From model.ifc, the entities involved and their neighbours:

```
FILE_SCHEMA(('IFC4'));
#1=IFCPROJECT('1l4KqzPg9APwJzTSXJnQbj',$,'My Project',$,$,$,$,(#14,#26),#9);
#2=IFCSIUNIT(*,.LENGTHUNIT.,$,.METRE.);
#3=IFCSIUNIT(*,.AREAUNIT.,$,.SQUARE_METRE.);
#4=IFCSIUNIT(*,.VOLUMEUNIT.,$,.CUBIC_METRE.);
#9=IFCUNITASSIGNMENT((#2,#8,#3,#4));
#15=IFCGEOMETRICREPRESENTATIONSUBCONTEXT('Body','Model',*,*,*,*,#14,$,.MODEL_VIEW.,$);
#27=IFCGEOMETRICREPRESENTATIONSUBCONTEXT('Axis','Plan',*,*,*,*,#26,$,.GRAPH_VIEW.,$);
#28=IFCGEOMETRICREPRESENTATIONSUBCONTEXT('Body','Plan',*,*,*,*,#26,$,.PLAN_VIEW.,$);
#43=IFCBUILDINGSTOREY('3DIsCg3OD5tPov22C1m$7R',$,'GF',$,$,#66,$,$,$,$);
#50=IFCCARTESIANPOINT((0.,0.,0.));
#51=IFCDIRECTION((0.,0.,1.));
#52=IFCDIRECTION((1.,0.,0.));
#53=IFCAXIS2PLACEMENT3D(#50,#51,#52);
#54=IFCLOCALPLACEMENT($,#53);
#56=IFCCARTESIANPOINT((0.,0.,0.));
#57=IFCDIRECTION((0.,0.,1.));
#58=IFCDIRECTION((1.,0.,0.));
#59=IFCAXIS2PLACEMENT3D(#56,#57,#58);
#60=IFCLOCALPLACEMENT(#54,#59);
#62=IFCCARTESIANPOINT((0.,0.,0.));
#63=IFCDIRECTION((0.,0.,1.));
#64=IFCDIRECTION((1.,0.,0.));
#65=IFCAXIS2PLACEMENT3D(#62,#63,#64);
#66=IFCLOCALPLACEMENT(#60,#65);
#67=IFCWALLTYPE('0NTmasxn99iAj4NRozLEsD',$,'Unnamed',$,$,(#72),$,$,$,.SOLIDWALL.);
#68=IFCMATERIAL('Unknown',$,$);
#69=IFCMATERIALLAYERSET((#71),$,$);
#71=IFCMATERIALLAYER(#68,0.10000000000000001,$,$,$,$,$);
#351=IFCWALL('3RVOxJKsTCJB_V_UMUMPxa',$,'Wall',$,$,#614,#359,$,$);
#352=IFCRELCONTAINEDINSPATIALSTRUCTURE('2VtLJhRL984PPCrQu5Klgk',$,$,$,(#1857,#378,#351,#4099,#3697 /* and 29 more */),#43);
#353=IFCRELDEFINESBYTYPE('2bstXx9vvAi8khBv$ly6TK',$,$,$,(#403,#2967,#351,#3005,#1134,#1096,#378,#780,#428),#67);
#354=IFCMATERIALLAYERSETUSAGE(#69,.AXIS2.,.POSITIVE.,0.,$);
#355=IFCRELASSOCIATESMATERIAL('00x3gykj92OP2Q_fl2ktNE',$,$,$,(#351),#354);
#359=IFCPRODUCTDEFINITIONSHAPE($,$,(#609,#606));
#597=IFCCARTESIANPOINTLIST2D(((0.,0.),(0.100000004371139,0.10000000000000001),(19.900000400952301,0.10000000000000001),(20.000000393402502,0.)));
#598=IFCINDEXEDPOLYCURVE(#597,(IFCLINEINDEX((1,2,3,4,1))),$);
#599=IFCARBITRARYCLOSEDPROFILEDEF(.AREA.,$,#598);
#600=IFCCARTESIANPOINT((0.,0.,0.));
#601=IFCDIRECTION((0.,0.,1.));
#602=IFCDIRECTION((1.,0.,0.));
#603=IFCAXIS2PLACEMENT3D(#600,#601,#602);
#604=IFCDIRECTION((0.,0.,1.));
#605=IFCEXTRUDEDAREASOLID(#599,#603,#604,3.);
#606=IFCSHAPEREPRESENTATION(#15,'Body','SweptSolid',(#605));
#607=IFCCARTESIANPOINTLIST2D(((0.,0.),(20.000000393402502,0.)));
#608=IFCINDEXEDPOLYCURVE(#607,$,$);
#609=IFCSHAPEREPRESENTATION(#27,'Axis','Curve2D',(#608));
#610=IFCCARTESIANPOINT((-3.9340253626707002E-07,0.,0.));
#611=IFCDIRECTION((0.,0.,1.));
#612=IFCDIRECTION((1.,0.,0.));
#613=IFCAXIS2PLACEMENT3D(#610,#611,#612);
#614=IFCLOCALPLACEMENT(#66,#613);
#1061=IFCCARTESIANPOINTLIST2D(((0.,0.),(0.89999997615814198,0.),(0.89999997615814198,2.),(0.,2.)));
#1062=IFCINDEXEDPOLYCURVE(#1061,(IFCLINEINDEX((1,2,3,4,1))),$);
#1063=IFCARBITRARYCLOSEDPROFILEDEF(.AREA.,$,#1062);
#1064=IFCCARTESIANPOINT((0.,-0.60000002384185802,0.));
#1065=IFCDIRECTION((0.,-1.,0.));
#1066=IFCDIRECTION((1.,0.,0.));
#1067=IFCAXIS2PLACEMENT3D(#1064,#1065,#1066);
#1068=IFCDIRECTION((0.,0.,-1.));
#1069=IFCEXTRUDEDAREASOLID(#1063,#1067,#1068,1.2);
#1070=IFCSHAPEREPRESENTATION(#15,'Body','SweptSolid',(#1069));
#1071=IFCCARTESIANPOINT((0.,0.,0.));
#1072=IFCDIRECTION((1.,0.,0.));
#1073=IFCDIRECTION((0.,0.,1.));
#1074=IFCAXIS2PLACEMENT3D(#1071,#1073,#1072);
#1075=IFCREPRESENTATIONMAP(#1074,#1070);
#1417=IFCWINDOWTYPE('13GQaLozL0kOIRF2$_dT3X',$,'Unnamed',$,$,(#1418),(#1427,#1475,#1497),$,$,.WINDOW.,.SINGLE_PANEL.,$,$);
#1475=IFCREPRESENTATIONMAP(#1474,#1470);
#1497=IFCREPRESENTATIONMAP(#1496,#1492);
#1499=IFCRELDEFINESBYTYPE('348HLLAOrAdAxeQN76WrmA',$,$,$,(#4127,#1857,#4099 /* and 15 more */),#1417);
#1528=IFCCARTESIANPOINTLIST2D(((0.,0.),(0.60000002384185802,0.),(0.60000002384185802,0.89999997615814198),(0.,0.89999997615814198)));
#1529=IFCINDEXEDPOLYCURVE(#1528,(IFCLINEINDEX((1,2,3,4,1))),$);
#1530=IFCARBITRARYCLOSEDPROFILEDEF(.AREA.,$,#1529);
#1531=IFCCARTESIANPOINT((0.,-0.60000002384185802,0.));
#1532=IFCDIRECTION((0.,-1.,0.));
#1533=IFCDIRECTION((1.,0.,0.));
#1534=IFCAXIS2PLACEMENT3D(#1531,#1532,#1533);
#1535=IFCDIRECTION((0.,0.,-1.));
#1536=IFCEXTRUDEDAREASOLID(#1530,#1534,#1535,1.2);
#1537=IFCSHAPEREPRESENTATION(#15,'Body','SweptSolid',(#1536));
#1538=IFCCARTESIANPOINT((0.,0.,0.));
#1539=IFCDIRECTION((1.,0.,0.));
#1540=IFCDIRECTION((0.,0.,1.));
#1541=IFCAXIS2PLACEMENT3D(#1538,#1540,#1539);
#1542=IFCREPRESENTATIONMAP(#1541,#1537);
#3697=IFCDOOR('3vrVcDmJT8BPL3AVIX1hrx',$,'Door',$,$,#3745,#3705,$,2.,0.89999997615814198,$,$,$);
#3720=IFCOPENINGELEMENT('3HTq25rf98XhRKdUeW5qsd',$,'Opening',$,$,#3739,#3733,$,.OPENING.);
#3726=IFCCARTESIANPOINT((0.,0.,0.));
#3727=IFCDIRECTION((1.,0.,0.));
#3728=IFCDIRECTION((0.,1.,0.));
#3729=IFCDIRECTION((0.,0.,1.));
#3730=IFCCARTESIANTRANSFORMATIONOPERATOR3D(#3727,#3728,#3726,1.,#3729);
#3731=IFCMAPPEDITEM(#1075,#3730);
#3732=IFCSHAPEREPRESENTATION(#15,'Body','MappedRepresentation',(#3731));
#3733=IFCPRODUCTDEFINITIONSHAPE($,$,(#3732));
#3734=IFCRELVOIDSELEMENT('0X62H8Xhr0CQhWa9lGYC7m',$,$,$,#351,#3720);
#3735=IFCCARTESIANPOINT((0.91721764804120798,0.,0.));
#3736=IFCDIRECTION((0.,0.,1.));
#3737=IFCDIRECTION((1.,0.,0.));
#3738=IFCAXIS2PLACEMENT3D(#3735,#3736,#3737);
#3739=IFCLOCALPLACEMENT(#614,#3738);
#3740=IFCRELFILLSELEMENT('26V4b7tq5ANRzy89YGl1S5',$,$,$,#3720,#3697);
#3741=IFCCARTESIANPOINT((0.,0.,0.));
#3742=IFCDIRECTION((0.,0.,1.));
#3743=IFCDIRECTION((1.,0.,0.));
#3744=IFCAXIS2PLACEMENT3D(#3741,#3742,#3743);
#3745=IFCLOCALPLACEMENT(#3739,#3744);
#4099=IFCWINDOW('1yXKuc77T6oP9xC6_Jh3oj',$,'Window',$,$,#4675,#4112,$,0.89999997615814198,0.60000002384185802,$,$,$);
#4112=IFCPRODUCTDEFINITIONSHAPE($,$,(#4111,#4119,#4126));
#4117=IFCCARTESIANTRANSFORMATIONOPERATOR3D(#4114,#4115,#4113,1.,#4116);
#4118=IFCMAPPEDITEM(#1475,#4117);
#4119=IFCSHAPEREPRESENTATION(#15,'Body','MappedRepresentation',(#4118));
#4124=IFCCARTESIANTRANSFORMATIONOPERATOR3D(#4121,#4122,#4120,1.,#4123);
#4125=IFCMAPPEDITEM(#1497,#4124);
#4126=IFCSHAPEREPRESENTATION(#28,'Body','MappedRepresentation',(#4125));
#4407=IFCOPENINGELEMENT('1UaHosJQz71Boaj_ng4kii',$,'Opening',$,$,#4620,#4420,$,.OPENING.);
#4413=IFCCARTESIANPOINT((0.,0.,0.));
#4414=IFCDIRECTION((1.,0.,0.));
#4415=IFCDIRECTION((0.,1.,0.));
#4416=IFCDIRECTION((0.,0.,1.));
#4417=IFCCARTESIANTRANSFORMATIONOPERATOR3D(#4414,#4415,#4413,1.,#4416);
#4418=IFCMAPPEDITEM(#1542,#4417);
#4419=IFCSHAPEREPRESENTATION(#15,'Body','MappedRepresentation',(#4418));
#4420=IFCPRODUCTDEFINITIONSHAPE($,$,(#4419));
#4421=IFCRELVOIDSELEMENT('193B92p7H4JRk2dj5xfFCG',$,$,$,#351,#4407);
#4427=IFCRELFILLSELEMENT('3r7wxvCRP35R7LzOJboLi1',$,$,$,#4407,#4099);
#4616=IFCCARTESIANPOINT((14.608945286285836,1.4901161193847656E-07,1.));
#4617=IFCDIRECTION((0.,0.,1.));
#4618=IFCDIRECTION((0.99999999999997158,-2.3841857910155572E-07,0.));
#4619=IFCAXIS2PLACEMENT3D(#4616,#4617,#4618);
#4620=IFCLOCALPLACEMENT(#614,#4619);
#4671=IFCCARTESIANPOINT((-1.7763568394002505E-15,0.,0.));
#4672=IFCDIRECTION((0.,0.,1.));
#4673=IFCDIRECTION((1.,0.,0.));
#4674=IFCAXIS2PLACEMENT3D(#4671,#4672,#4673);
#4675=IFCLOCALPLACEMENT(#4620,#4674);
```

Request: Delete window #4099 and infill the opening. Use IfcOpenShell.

```python
import ifcopenshell
import ifcopenshell.api.feature
import ifcopenshell.api.root
import ifcopenshell.geom
import ifcopenshell.util.shape

model = ifcopenshell.open("model.ifc")
settings = ifcopenshell.geom.settings()


def volume(element):
    """Net volume in cubic metres, openings subtracted."""
    shape = ifcopenshell.geom.create_shape(settings, element)
    return ifcopenshell.util.shape.get_volume(shape.geometry)


window = model.by_guid("1yXKuc77T6oP9xC6_Jh3oj")
opening = window.FillsVoids[0].RelatingOpeningElement
wall = opening.VoidsElements[0].RelatingBuildingElement
before = volume(wall)

ifcopenshell.api.root.remove_product(model, product=window)
ifcopenshell.api.feature.remove_feature(model, feature=opening)

after = volume(wall)

print(f"wall volume {before:.3f} -> {after:.3f} m3")

model.write("model_updated.ifc")
```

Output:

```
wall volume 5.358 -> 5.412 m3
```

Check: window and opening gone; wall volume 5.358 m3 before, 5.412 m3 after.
